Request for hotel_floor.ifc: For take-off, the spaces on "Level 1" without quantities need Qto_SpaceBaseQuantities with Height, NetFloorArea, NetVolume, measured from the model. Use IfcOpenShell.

First a look at what the model holds.

```python
import ifcopenshell
import ifcopenshell.util.element
import ifcopenshell.util.unit

model = ifcopenshell.open("hotel_floor.ifc")
print(model.schema)
for unit_type in ("LENGTHUNIT", "AREAUNIT", "VOLUMEUNIT"):
    print(unit_type, ifcopenshell.util.unit.calculate_unit_scale(model, unit_type))
storey = next(s for s in model.by_type("IfcBuildingStorey") if s.Name == "Level 1")
spaces = [e for e in ifcopenshell.util.element.get_decomposition(storey) if e.is_a("IfcSpace")]
for e in sorted(spaces, key=lambda e: e.id()):
    print(e.id(), e.is_a(), e.Name, list(ifcopenshell.util.element.get_psets(e, qtos_only=True)), sep=" | ")
```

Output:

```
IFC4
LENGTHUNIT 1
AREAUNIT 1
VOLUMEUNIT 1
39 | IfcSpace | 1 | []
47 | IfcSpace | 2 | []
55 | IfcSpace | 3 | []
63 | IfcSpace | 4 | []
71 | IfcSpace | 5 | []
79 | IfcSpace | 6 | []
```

```python
import ifcopenshell
import ifcopenshell.api.pset
import ifcopenshell.geom
import ifcopenshell.util.element
import ifcopenshell.util.shape
import ifcopenshell.util.unit

model = ifcopenshell.open("hotel_floor.ifc")
unit_scale = ifcopenshell.util.unit.calculate_unit_scale(model)
area_scale = ifcopenshell.util.unit.calculate_unit_scale(model, "AREAUNIT")
volume_scale = ifcopenshell.util.unit.calculate_unit_scale(model, "VOLUMEUNIT")
settings = ifcopenshell.geom.settings()

storey = next(s for s in model.by_type("IfcBuildingStorey") if s.Name == "Level 1")
spaces = [e for e in ifcopenshell.util.element.get_decomposition(storey) if e.is_a("IfcSpace")]

for e in sorted(spaces, key=lambda e: e.id()):
    if ifcopenshell.util.element.get_psets(e, qtos_only=True, should_inherit=False):
        continue
    # Geometry comes back in metres, in the element's own axes.
    shape = ifcopenshell.geom.create_shape(settings, e)
    values = {
        "Height": ifcopenshell.util.shape.get_z(shape.geometry) / unit_scale,
        "NetFloorArea": ifcopenshell.util.shape.get_footprint_area(shape.geometry) / area_scale,
        "NetVolume": ifcopenshell.util.shape.get_volume(shape.geometry) / volume_scale,
    }
    qto = ifcopenshell.api.pset.add_qto(model, product=e, name="Qto_SpaceBaseQuantities")
    ifcopenshell.api.pset.edit_qto(model, qto=qto, properties=values)
    print(e.id(), {k: round(v, 3) for k, v in values.items()})

model.write("hotel_floor_v2.ifc")
```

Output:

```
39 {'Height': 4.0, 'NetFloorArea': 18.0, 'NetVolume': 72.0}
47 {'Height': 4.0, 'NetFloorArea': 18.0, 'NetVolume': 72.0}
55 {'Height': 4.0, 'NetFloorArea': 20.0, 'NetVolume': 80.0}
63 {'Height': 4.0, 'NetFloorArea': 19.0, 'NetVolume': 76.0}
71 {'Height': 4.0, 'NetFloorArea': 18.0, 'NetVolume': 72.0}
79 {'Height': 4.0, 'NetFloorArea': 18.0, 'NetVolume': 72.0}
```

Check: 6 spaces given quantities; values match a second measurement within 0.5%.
